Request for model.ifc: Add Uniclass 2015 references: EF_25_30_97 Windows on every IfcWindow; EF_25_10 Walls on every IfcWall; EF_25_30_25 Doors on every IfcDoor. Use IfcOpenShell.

First a look at what the model holds.

```python
import ifcopenshell

model = ifcopenshell.open("model.ifc")
print(model.schema)
print("classifications:", [c.Name for c in model.by_type("IfcClassification")])
for ifc_class in ("IfcDoor", "IfcRoof", "IfcStair", "IfcWall", "IfcWindow"):
    print(ifc_class, len(model.by_type(ifc_class)))
```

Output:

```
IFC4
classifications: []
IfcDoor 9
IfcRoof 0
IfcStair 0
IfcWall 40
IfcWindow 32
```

```python
import ifcopenshell
import ifcopenshell.api.classification

model = ifcopenshell.open("model.ifc")

system = ifcopenshell.api.classification.add_classification(model, classification="Uniclass 2015")

codes = {
    "IfcWindow": ("EF_25_30_97", "Windows"),
    "IfcWall": ("EF_25_10", "Walls"),
    "IfcDoor": ("EF_25_30_25", "Doors"),
}
for ifc_class, (code, name) in codes.items():
    products = model.by_type(ifc_class)
    ifcopenshell.api.classification.add_reference(
        model, products=products, classification=system, identification=code, name=name
    )
    print(code, len(products))

model.write("model-out.ifc")
```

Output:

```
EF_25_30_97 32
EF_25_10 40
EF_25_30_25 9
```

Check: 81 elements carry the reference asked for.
